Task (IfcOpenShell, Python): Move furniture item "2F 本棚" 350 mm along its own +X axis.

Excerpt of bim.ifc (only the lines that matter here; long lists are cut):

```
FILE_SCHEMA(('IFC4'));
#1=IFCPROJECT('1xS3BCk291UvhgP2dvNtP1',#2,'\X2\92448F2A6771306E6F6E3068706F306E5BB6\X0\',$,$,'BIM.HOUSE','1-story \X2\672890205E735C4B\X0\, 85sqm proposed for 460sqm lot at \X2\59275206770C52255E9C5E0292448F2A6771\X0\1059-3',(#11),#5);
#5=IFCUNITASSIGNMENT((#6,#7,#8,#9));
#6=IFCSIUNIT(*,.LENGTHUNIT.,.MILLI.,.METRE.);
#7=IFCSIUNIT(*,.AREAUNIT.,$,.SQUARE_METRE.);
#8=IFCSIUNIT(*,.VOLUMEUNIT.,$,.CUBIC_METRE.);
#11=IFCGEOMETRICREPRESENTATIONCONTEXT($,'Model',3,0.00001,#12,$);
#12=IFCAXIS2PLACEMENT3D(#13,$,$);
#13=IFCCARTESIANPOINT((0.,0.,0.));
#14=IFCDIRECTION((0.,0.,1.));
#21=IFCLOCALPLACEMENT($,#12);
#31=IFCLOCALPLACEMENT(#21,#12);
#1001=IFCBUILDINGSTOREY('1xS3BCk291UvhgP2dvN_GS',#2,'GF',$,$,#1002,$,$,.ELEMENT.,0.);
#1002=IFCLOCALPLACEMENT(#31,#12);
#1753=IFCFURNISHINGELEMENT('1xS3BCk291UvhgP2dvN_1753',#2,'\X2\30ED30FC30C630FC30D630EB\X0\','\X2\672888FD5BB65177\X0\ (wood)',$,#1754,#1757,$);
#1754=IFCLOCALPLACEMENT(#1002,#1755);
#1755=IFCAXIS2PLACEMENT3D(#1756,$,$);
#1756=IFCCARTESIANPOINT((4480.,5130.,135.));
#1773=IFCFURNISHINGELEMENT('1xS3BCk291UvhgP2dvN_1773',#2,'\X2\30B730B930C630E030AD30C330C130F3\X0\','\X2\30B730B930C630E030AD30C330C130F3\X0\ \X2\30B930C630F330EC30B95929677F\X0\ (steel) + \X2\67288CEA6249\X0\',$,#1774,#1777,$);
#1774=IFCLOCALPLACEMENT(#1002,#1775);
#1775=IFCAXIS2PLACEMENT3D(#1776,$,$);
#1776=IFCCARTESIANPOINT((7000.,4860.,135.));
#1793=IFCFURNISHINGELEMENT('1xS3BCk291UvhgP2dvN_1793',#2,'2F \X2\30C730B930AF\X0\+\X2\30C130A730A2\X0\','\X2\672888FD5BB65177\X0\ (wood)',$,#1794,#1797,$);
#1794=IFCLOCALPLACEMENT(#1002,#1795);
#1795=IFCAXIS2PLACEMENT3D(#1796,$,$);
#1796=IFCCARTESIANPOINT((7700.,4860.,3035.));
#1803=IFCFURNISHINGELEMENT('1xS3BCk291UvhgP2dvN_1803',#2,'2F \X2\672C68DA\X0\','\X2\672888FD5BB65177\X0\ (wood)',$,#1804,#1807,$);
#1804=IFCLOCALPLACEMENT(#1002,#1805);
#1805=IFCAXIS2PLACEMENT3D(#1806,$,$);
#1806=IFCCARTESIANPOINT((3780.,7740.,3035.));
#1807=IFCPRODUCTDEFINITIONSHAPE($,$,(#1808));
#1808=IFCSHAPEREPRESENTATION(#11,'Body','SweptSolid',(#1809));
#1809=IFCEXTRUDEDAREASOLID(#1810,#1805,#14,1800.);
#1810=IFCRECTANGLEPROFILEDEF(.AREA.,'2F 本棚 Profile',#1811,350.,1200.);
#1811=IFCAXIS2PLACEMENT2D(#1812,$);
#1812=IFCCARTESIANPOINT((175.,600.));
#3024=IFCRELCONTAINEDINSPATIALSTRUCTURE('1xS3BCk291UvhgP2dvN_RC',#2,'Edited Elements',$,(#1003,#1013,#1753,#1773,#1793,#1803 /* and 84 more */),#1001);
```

```python
import ifcopenshell
import ifcopenshell.api.geometry
import ifcopenshell.util.placement
import ifcopenshell.util.unit

model = ifcopenshell.open("bim.ifc")
unit_scale = ifcopenshell.util.unit.calculate_unit_scale(model)

item = model.by_guid("1xS3BCk291UvhgP2dvN_1803")
matrix = ifcopenshell.util.placement.get_local_placement(item.ObjectPlacement)
matrix[:3, 3] += matrix[:3, 0] * 0.35 / unit_scale
ifcopenshell.api.geometry.edit_object_placement(model, product=item, matrix=matrix, is_si=False)

print(ifcopenshell.util.placement.get_local_placement(item.ObjectPlacement).round(3) + 0.0)

model.write("bim_v2.ifc")
```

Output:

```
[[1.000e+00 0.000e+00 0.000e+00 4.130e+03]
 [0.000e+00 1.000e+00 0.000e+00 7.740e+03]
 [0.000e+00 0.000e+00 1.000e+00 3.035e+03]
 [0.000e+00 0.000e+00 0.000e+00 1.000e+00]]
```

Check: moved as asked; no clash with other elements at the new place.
